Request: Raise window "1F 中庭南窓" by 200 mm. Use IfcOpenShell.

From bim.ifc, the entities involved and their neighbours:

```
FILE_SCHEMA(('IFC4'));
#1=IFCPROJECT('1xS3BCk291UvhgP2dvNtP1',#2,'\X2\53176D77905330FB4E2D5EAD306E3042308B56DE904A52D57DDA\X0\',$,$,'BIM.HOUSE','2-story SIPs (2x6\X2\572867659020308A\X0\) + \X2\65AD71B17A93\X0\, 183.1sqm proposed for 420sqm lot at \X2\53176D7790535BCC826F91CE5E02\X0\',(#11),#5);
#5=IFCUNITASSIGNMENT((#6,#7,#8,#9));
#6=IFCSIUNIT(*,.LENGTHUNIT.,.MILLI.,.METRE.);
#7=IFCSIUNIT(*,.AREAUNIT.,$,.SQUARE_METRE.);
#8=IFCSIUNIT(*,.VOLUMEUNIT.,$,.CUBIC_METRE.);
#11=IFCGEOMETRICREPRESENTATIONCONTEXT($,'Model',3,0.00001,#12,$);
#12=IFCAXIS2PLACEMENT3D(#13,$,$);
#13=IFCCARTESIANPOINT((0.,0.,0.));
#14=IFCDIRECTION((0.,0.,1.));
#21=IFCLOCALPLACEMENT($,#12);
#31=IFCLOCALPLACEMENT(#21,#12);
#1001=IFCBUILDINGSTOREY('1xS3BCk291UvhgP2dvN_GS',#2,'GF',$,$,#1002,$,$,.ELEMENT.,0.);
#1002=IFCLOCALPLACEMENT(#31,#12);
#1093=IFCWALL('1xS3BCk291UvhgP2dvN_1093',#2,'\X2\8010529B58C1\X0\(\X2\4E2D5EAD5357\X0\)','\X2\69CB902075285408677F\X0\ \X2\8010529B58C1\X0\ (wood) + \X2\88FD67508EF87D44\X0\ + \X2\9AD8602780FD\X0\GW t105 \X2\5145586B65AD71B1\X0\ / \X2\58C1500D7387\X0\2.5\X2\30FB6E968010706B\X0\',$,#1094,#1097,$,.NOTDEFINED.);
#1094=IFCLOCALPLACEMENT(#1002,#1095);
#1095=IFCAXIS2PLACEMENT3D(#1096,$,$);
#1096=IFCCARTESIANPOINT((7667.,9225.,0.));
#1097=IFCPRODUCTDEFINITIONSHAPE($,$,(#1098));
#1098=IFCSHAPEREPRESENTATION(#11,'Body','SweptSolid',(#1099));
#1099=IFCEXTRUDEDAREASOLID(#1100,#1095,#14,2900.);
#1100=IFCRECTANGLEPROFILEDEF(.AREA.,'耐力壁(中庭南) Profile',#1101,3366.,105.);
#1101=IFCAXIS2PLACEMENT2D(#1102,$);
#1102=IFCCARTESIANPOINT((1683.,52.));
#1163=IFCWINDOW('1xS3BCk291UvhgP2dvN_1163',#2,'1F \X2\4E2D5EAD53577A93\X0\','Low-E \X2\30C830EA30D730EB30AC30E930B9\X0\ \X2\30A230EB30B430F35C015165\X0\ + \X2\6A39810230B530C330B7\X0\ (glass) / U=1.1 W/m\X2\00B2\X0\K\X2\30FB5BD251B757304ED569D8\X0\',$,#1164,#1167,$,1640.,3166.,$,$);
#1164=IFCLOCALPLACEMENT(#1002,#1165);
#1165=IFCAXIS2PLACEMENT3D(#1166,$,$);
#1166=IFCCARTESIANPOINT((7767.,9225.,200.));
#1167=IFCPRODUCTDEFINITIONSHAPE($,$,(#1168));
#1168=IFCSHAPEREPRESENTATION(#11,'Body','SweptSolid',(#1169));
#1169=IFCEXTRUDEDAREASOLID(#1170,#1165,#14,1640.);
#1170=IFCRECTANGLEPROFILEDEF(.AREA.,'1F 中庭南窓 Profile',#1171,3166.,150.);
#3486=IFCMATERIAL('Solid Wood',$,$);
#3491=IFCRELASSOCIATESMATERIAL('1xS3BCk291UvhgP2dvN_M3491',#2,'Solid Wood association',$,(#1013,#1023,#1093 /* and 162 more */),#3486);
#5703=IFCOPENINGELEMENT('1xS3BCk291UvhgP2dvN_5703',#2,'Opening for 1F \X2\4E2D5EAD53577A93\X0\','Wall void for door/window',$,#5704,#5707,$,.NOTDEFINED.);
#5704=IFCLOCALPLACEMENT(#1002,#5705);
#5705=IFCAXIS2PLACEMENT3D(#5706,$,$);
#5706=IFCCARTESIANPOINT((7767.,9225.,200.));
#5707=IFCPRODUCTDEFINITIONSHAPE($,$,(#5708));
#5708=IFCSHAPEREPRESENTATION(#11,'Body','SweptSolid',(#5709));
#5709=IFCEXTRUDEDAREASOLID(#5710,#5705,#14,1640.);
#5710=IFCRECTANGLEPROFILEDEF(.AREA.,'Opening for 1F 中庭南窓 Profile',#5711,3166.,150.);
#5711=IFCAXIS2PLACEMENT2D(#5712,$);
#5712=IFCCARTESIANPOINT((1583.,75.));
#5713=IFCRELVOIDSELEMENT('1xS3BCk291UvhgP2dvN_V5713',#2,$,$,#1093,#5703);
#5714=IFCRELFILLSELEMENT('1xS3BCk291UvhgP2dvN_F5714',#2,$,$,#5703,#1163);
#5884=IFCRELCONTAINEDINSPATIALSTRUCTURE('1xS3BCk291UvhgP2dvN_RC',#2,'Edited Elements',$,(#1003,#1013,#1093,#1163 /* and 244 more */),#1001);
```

```python
import numpy as np
import ifcopenshell
import ifcopenshell.api.geometry
import ifcopenshell.util.placement
import ifcopenshell.util.unit

model = ifcopenshell.open("bim.ifc")
unit_scale = ifcopenshell.util.unit.calculate_unit_scale(model)

window = model.by_guid("1xS3BCk291UvhgP2dvN_1163")
opening = window.FillsVoids[0].RelatingOpeningElement
dz = 200.0

shift = np.array([0.0, 0.0, dz])
# The window is not placed relative to its opening, so move both.
for product in (opening, window):
    matrix = ifcopenshell.util.placement.get_local_placement(product.ObjectPlacement)
    matrix[:3, 3] += shift
    ifcopenshell.api.geometry.edit_object_placement(model, product=product, matrix=matrix, is_si=False)

print(f"moved by {dz * unit_scale:+.3f} m")

model.write("bim-out.ifc")
```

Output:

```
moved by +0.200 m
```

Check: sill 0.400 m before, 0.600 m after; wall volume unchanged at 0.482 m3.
